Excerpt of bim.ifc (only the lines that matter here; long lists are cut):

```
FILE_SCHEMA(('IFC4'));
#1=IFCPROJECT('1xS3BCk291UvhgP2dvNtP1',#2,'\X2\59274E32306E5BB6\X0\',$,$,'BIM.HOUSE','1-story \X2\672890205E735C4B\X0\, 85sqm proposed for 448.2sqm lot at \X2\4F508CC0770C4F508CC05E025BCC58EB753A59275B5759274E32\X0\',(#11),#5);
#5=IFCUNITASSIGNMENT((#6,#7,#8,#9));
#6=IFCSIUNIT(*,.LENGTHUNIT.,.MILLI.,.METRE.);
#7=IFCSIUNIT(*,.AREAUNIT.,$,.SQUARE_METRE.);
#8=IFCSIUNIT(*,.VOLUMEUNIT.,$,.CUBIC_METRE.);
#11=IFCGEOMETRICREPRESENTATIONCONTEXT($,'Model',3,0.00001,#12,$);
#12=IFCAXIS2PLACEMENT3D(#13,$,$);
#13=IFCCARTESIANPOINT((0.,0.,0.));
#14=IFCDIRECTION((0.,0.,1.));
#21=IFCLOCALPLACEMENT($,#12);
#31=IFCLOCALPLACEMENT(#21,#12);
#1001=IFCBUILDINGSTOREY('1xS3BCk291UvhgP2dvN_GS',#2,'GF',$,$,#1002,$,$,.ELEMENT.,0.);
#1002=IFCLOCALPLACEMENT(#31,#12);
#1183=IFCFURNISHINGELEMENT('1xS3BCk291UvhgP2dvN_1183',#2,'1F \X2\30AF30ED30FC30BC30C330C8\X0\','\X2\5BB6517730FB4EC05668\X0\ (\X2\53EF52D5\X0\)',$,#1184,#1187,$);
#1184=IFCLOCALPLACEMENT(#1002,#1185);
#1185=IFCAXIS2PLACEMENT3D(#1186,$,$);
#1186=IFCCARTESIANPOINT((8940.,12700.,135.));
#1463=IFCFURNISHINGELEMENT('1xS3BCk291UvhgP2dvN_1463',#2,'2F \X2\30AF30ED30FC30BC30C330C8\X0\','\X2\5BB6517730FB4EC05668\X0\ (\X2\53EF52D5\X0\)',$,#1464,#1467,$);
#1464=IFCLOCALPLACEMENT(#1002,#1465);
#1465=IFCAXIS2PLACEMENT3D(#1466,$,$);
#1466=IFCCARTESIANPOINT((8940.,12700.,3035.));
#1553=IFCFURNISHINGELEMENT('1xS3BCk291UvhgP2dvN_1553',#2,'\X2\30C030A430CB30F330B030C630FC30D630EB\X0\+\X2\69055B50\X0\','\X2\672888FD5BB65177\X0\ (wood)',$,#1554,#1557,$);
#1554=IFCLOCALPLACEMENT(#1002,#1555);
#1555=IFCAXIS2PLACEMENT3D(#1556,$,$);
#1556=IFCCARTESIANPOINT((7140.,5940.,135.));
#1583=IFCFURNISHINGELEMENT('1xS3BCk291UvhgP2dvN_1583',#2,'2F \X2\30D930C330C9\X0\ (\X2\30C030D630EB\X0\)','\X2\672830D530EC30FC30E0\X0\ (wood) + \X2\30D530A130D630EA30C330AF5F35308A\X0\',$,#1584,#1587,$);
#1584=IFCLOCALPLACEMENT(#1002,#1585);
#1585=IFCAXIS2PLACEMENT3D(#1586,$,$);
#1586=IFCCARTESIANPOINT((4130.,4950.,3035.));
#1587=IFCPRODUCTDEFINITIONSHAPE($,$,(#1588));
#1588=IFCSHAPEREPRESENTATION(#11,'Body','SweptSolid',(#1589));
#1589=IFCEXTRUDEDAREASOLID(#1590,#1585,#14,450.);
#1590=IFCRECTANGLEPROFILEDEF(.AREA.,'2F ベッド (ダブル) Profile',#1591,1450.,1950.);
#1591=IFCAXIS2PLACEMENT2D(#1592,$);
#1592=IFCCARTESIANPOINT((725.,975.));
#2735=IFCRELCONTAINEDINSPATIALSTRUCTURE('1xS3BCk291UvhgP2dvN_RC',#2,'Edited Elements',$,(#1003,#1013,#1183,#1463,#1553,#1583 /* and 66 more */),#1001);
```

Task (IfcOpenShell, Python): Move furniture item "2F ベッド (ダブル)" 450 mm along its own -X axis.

```python
import ifcopenshell
import ifcopenshell.api.geometry
import ifcopenshell.util.placement
import ifcopenshell.util.unit

model = ifcopenshell.open("bim.ifc")
unit_scale = ifcopenshell.util.unit.calculate_unit_scale(model)

item = model.by_id(1583)
matrix = ifcopenshell.util.placement.get_local_placement(item.ObjectPlacement)
matrix[:3, 3] -= matrix[:3, 0] * 0.45 / unit_scale
ifcopenshell.api.geometry.edit_object_placement(model, product=item, matrix=matrix, is_si=False)

print(ifcopenshell.util.placement.get_local_placement(item.ObjectPlacement).round(3) + 0.0)

model.write("bim_rev.ifc")
```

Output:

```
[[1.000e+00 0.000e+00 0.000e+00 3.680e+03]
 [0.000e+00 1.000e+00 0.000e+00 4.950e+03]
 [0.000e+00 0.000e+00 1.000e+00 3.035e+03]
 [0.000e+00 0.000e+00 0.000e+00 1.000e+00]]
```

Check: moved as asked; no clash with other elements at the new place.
